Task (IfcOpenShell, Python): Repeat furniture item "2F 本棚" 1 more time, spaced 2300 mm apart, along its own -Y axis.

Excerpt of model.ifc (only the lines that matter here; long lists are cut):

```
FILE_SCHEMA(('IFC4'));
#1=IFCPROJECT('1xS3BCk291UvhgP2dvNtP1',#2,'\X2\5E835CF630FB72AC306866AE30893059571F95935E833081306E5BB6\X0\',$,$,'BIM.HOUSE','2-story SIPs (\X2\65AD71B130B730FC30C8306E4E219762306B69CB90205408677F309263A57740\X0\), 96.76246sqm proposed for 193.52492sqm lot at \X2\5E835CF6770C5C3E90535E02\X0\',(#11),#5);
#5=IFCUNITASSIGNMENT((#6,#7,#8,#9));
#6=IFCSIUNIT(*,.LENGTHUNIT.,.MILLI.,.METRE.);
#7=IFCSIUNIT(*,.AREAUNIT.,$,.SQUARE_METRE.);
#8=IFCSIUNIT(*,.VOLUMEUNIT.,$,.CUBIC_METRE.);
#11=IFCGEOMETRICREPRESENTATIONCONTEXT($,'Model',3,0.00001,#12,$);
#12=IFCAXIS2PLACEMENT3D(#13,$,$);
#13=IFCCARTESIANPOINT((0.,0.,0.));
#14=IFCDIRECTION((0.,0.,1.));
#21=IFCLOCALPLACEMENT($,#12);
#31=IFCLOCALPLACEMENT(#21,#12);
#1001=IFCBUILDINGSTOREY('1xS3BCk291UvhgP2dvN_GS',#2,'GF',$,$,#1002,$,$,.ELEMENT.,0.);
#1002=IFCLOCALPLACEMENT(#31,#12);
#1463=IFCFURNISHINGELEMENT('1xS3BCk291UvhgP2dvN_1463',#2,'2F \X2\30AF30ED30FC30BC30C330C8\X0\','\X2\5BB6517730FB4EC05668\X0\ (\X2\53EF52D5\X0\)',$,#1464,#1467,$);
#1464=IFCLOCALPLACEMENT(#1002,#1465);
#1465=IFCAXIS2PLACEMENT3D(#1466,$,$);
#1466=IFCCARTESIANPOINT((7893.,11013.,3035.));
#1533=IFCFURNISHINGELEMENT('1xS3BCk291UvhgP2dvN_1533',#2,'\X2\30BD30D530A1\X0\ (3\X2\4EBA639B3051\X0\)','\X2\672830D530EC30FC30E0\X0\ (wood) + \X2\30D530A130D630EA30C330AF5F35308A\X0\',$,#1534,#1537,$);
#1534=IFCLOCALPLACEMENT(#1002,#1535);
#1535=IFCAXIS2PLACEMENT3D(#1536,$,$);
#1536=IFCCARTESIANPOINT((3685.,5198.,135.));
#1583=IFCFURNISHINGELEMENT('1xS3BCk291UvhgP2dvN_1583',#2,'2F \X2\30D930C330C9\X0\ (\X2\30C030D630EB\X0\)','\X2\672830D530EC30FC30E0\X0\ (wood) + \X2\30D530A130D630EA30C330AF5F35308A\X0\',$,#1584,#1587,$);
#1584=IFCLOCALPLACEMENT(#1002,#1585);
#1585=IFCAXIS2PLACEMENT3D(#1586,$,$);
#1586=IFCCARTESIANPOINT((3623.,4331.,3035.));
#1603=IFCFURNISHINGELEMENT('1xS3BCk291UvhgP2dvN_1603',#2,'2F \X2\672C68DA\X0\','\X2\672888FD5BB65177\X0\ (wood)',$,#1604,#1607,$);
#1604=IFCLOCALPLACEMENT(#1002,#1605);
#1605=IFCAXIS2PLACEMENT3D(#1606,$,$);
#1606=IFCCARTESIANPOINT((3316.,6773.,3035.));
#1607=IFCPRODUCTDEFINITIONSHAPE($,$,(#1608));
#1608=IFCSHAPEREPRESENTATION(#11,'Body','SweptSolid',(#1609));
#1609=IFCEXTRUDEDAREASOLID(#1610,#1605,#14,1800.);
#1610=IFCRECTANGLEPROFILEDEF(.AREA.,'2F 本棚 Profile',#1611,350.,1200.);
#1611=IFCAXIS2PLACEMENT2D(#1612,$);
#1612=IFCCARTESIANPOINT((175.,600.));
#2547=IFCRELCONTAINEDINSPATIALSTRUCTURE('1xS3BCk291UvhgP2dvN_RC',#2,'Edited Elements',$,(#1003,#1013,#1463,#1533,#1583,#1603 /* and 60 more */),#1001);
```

```python
import ifcopenshell
import ifcopenshell.api.geometry
import ifcopenshell.api.root
import ifcopenshell.util.element
import ifcopenshell.util.placement

model = ifcopenshell.open("model.ifc")


def reuse_history(source, copy):
    """copy_class also copies each property set's owner history, people and application; keep the originals."""
    for rel in copy.IsDefinedBy:
        if rel.is_a("IfcRelDefinesByProperties") and (history := rel.RelatingPropertyDefinition.OwnerHistory):
            rel.RelatingPropertyDefinition.OwnerHistory = source.OwnerHistory
            ifcopenshell.util.element.remove_deep2(model, history)


source = model.by_id(1603)
base = ifcopenshell.util.placement.get_local_placement(source.ObjectPlacement)
step = -base[:3, 1] * 2300.0

for i in range(1, 2):
    copy = ifcopenshell.api.root.copy_class(model, product=source)
    copy.Representation = ifcopenshell.util.element.copy_deep(
        model, source.Representation, exclude=["IfcGeometricRepresentationContext", "IfcRepresentationMap"]
    )
    reuse_history(source, copy)
    matrix = base.copy()
    matrix[:3, 3] += i * step
    print("added at", matrix[:3, 3].round(3) + 0.0)
    ifcopenshell.api.geometry.edit_object_placement(model, product=copy, matrix=matrix, is_si=False)

model.write("model_updated.ifc")
```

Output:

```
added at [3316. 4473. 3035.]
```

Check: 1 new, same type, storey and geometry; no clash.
